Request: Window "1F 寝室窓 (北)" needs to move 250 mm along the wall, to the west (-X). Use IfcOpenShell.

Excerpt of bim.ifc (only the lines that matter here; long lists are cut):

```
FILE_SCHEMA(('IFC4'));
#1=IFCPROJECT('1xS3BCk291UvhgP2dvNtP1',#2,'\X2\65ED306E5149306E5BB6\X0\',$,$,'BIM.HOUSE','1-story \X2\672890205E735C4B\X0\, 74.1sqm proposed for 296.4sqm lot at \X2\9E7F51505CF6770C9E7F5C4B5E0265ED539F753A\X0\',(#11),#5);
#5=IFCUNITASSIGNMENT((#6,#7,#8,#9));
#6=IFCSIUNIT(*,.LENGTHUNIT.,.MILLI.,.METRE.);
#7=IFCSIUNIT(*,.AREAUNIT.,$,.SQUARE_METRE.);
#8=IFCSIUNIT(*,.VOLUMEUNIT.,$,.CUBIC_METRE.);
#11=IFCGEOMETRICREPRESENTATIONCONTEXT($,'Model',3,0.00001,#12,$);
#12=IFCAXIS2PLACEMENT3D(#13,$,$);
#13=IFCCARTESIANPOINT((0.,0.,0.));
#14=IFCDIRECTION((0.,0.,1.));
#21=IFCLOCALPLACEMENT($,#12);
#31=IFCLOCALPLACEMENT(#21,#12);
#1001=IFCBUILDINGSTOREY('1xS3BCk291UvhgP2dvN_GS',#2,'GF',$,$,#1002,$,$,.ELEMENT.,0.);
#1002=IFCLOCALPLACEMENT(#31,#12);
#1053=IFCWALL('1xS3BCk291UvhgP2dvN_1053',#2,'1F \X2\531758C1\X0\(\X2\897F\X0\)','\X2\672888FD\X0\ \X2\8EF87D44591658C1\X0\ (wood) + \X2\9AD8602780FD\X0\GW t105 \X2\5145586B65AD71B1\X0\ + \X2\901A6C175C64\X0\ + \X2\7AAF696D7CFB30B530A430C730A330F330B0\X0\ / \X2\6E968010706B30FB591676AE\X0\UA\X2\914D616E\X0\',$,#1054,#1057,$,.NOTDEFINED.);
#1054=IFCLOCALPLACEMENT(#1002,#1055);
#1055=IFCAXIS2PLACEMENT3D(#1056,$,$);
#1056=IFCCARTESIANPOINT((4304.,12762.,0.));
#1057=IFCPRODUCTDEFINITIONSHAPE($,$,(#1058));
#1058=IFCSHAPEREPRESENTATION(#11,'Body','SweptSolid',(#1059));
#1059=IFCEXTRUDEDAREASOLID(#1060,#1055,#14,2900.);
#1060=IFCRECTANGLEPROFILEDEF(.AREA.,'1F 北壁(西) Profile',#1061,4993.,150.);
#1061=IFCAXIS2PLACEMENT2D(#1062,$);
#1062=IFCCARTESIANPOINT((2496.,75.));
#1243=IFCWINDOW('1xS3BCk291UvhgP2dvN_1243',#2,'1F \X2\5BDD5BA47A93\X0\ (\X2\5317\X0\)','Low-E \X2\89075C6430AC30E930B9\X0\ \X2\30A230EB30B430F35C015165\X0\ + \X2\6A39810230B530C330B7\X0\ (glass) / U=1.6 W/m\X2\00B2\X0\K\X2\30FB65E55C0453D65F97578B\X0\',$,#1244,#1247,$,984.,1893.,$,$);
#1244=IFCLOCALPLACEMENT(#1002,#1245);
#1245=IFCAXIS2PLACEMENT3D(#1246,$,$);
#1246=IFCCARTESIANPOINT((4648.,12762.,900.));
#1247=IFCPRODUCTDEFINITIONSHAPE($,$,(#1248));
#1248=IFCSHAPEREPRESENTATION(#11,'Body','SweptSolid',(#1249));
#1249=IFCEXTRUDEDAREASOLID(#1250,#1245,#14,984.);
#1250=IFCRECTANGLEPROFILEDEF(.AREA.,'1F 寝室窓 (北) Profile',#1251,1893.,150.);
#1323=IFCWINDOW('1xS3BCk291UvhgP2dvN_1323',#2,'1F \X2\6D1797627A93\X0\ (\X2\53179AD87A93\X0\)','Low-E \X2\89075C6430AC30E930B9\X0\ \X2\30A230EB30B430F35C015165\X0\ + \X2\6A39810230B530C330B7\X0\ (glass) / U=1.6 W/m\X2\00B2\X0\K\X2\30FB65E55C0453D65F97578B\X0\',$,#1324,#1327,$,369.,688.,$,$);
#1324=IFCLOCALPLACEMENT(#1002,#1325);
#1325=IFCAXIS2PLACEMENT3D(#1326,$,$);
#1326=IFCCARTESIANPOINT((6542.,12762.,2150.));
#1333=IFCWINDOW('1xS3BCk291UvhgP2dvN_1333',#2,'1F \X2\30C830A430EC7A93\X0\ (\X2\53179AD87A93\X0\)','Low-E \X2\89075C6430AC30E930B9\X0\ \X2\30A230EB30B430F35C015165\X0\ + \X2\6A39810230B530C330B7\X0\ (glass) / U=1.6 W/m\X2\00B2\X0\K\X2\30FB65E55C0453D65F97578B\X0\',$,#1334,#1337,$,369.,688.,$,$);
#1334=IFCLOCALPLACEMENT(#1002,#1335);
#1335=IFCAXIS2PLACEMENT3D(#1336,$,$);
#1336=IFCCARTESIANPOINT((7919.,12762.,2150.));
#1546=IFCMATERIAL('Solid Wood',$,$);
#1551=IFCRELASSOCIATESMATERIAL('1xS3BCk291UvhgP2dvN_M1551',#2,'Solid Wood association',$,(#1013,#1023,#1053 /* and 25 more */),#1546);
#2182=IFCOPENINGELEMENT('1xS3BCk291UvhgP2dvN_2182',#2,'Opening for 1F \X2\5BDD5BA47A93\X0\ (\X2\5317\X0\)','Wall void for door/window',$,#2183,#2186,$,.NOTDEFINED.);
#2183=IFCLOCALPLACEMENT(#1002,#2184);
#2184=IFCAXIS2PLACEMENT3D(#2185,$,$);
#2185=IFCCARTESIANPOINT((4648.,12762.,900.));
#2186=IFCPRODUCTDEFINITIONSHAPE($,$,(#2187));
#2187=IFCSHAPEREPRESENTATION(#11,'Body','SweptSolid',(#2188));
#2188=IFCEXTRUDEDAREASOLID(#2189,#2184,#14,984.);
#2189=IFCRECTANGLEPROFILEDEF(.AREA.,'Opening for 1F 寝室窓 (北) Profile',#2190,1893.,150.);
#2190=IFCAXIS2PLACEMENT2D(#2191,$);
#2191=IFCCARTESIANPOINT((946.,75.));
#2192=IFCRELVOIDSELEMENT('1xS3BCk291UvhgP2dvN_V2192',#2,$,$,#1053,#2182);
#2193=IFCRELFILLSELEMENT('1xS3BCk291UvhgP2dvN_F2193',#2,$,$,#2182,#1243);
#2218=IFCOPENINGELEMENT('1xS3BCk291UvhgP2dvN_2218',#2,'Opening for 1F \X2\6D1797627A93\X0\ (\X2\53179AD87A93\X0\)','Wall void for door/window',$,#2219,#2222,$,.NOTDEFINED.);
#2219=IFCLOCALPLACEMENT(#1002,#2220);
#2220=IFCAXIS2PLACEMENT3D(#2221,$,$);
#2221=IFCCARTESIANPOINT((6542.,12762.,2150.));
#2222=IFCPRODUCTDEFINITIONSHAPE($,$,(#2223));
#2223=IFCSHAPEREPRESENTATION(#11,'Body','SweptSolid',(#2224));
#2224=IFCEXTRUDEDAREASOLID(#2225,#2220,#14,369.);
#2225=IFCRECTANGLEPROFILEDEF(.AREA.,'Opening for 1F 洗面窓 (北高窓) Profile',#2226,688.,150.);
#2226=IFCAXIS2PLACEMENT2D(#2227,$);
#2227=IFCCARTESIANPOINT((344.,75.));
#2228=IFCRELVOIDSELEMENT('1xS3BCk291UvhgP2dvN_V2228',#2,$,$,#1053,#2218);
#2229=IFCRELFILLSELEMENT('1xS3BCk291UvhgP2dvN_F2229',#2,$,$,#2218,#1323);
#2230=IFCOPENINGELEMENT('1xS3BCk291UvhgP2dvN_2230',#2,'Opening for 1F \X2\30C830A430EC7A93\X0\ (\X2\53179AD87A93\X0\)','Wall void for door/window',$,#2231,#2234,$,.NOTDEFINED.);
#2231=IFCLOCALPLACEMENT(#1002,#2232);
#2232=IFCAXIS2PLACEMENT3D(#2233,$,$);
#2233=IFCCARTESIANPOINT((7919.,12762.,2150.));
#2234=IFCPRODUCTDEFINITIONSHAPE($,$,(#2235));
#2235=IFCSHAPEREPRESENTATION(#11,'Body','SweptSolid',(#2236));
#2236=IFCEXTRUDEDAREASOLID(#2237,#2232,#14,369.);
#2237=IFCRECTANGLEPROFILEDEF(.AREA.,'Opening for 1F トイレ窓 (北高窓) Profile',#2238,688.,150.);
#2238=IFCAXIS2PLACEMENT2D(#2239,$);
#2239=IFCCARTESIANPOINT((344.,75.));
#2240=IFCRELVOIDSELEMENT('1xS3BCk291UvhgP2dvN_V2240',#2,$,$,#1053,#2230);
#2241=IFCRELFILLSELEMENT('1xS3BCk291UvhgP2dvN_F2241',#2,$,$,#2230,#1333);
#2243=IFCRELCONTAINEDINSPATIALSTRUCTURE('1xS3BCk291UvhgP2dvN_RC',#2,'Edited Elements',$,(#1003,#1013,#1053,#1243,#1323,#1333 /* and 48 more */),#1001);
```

```python
import ifcopenshell
import ifcopenshell.api.geometry
import ifcopenshell.util.placement
import ifcopenshell.util.unit

model = ifcopenshell.open("bim.ifc")
unit_scale = ifcopenshell.util.unit.calculate_unit_scale(model)

window = model.by_guid("1xS3BCk291UvhgP2dvN_1243")
opening = window.FillsVoids[0].RelatingOpeningElement
wall = opening.VoidsElements[0].RelatingBuildingElement

wall_matrix = ifcopenshell.util.placement.get_local_placement(wall.ObjectPlacement)
shift = wall_matrix[:3, 0] * -0.25 / unit_scale
before = ifcopenshell.util.placement.get_local_placement(window.ObjectPlacement)[:3, 3].copy()

# The window is not placed relative to its opening, so move both.
for product in (opening, window):
    matrix = ifcopenshell.util.placement.get_local_placement(product.ObjectPlacement)
    matrix[:3, 3] += shift
    ifcopenshell.api.geometry.edit_object_placement(model, product=product, matrix=matrix, is_si=False)

after = ifcopenshell.util.placement.get_local_placement(window.ObjectPlacement)[:3, 3]
print("window moved by", (after - before).round(3) + 0.0)

model.write("bim_rev.ifc")
```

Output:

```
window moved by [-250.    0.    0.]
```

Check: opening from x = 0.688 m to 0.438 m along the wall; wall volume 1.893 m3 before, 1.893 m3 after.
